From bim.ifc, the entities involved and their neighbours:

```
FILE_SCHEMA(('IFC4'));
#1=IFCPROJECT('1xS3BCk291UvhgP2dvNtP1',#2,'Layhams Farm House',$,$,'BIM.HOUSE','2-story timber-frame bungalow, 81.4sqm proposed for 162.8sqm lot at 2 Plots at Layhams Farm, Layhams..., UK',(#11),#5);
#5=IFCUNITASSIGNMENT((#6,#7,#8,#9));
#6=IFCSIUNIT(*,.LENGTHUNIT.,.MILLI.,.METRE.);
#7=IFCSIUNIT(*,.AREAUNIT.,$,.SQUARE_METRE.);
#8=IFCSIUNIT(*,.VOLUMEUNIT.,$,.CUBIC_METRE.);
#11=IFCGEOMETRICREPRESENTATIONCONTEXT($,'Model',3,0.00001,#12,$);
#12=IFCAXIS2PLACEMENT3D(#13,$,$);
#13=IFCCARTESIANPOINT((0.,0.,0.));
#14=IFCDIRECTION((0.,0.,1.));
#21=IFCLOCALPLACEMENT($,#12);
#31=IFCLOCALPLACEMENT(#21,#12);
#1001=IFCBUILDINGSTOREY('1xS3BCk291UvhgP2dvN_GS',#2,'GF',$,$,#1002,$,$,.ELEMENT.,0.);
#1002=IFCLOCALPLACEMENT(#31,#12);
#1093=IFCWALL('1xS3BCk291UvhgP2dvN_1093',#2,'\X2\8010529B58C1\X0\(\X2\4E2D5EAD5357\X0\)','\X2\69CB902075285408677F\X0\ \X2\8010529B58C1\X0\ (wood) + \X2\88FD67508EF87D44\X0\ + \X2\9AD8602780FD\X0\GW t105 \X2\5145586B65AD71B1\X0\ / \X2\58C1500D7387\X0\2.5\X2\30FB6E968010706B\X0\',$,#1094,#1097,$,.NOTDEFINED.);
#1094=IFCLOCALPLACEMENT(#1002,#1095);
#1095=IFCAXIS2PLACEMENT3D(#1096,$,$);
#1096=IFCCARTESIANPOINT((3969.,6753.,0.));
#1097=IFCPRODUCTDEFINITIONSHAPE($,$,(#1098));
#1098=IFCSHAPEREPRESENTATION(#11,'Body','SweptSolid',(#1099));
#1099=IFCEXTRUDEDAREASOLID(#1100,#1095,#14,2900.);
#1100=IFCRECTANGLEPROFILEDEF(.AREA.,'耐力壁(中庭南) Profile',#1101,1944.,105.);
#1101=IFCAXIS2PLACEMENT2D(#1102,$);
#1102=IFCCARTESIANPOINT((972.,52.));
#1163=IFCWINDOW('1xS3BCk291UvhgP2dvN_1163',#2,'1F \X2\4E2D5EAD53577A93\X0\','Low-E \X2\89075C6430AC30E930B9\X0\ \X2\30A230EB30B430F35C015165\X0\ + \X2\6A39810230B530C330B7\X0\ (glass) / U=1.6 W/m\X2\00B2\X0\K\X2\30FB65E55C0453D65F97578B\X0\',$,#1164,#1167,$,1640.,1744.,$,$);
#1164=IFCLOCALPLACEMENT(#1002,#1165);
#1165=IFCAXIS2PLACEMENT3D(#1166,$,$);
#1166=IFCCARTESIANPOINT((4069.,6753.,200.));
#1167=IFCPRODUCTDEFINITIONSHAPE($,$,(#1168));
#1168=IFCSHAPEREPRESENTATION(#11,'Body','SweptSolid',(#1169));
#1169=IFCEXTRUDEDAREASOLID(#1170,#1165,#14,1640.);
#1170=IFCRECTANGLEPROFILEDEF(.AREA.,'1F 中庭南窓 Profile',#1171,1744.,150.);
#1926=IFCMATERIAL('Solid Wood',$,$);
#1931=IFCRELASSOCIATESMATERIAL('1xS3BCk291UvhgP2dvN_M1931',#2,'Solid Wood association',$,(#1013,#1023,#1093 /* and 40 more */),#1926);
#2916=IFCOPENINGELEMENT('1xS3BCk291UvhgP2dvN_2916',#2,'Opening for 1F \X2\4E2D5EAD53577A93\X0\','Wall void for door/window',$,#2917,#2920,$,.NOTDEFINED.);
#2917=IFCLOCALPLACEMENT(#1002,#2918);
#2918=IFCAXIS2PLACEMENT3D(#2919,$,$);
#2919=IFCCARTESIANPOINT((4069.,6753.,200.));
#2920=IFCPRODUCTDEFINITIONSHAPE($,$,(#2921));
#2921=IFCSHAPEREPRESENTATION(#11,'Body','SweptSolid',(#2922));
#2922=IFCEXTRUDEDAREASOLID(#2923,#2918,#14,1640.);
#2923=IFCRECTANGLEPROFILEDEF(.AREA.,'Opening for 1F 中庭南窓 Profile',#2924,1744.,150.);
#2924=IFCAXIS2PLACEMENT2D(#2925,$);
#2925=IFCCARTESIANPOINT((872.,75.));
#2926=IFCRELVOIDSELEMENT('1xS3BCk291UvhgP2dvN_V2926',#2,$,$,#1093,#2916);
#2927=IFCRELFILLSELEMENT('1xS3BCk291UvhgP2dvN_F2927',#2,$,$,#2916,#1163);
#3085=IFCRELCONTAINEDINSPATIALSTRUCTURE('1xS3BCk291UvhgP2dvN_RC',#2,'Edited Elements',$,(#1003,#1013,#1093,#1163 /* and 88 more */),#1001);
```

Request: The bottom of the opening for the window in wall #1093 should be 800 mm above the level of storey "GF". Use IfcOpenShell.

```python
import numpy as np
import ifcopenshell
import ifcopenshell.api.geometry
import ifcopenshell.geom
import ifcopenshell.util.element
import ifcopenshell.util.placement
import ifcopenshell.util.shape
import ifcopenshell.util.unit

model = ifcopenshell.open("bim.ifc")
unit_scale = ifcopenshell.util.unit.calculate_unit_scale(model)

window = model.by_guid("1xS3BCk291UvhgP2dvN_1163")
opening = window.FillsVoids[0].RelatingOpeningElement
storey = ifcopenshell.util.element.get_container(window, ifc_class="IfcBuildingStorey")
level = ifcopenshell.util.placement.get_local_placement(storey.ObjectPlacement)[2, 3]

# The opening's origin need not be at the sill, so measure its lowest point.
shape = ifcopenshell.geom.create_shape(ifcopenshell.geom.settings(), opening)
bottom = ifcopenshell.util.shape.get_shape_bottom_elevation(shape, shape.geometry) / unit_scale
dz = level + 0.8 / unit_scale - bottom

shift = np.array([0.0, 0.0, dz])
# The window is not placed relative to its opening, so move both.
for product in (opening, window):
    matrix = ifcopenshell.util.placement.get_local_placement(product.ObjectPlacement)
    matrix[:3, 3] += shift
    ifcopenshell.api.geometry.edit_object_placement(model, product=product, matrix=matrix, is_si=False)

print(f"moved by {dz * unit_scale:+.3f} m")

model.write("bim_rev.ifc")
```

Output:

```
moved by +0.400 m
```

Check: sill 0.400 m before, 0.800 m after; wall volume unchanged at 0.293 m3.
